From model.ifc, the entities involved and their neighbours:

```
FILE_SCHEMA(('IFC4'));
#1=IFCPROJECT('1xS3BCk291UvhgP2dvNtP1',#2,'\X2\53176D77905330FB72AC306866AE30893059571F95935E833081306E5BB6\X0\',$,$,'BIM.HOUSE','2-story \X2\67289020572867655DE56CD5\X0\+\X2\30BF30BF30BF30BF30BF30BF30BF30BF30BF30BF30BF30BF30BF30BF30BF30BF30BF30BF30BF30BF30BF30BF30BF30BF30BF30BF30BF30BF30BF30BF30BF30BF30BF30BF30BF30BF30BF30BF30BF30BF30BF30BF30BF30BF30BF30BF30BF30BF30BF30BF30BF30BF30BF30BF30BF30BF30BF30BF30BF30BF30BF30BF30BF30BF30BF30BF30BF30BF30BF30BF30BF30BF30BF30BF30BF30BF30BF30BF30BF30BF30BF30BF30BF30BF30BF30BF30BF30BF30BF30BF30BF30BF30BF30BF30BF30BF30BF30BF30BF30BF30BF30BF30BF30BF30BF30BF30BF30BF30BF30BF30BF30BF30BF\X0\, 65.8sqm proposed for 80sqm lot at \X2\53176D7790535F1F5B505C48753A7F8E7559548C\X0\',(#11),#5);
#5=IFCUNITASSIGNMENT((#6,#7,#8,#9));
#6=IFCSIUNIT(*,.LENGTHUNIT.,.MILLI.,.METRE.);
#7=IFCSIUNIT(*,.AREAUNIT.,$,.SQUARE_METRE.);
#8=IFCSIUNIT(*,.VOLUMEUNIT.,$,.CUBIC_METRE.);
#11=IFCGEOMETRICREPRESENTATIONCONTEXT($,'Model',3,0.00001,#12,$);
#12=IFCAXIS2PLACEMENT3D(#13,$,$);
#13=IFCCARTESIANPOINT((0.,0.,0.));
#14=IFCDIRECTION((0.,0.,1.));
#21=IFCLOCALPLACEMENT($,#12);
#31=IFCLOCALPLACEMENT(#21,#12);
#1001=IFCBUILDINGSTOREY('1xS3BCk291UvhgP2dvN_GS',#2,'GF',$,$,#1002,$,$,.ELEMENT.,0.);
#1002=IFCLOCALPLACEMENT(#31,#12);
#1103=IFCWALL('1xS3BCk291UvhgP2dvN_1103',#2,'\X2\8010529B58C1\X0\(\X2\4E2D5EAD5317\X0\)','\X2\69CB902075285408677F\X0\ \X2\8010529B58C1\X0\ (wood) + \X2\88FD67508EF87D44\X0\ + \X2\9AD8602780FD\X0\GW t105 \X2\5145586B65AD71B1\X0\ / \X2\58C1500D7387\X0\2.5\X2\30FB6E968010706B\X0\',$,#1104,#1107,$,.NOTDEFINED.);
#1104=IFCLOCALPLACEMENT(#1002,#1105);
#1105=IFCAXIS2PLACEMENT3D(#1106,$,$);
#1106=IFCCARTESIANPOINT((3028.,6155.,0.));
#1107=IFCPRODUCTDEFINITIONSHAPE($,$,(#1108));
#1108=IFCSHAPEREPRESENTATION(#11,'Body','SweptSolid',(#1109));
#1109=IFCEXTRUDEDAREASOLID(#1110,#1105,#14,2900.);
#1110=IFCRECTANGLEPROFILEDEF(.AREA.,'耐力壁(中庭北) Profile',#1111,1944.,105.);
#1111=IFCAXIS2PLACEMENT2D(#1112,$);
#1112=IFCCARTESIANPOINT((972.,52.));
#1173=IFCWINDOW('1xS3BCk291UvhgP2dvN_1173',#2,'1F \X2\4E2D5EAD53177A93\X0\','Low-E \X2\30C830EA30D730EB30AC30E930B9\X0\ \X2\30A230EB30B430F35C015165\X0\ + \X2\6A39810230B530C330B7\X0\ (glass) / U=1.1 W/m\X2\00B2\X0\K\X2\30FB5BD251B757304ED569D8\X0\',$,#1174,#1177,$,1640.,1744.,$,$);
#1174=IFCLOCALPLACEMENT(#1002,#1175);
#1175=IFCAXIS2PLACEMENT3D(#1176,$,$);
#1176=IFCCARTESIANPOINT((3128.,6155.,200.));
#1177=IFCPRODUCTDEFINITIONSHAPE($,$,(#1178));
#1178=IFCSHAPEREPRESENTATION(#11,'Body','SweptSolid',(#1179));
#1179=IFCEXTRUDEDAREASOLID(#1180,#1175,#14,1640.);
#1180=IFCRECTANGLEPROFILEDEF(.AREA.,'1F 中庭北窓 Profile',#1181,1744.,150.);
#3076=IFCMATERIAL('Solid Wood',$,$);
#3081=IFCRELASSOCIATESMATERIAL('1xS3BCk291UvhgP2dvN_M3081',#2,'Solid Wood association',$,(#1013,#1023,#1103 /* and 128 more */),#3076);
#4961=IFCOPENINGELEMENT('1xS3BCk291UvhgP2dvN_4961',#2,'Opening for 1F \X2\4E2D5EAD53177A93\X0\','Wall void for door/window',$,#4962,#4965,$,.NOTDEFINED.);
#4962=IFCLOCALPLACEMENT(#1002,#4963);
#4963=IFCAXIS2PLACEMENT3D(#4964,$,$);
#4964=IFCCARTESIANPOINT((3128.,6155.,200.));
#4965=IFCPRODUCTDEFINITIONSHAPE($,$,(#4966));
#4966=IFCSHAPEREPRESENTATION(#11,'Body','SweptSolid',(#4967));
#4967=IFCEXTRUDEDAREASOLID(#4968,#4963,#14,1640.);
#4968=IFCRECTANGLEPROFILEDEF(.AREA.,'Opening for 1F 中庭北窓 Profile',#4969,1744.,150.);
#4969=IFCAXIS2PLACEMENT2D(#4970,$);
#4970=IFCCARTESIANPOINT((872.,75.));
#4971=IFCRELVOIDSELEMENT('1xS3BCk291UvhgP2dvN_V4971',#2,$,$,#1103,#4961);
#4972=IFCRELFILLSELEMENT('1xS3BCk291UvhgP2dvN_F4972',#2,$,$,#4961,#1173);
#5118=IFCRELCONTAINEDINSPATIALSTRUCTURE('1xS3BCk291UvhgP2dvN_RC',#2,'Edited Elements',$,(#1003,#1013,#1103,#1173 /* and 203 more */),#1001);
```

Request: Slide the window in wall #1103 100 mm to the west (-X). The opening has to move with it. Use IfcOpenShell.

```python
import ifcopenshell
import ifcopenshell.api.geometry
import ifcopenshell.util.placement
import ifcopenshell.util.unit

model = ifcopenshell.open("model.ifc")
unit_scale = ifcopenshell.util.unit.calculate_unit_scale(model)

window = model.by_guid("1xS3BCk291UvhgP2dvN_1173")
opening = window.FillsVoids[0].RelatingOpeningElement
wall = opening.VoidsElements[0].RelatingBuildingElement

wall_matrix = ifcopenshell.util.placement.get_local_placement(wall.ObjectPlacement)
shift = wall_matrix[:3, 0] * -0.1 / unit_scale
before = ifcopenshell.util.placement.get_local_placement(window.ObjectPlacement)[:3, 3].copy()

# The window is not placed relative to its opening, so move both.
for product in (opening, window):
    matrix = ifcopenshell.util.placement.get_local_placement(product.ObjectPlacement)
    matrix[:3, 3] += shift
    ifcopenshell.api.geometry.edit_object_placement(model, product=product, matrix=matrix, is_si=False)

after = ifcopenshell.util.placement.get_local_placement(window.ObjectPlacement)[:3, 3]
print("window moved by", (after - before).round(3) + 0.0)

model.write("model-out.ifc")
```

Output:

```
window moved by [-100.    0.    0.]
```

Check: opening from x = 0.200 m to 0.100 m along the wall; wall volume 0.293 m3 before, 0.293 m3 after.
